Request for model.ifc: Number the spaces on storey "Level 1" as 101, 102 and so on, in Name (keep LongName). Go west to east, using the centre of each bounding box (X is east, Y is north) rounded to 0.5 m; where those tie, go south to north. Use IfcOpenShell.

First a look at what the model holds.

```python
import ifcopenshell
import ifcopenshell.util.element
import ifcopenshell.util.placement

model = ifcopenshell.open("model.ifc")
print(model.schema)
storey = next(s for s in model.by_type("IfcBuildingStorey") if s.Name == "Level 1")
spaces = [e for e in ifcopenshell.util.element.get_decomposition(storey) if e.is_a("IfcSpace")]
for e in sorted(spaces, key=lambda e: e.id()):
    origin = ifcopenshell.util.placement.get_local_placement(e.ObjectPlacement)[:3, 3]
    print(e.id(), e.Name, e.LongName, origin.round(2) + 0.0, sep=" | ")
```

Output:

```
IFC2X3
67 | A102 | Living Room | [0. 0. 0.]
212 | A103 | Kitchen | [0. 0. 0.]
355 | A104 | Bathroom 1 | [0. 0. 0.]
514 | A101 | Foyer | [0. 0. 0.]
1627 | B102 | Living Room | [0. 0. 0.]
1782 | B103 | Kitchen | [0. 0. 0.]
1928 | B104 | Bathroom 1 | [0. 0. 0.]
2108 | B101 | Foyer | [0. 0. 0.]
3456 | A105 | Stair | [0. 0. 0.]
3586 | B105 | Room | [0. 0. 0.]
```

```python
import ifcopenshell
import ifcopenshell.geom
import ifcopenshell.util.element
import ifcopenshell.util.shape

model = ifcopenshell.open("model.ifc")
settings = ifcopenshell.geom.settings()
settings.set("use-world-coords", True)


def centre(element):
    shape = ifcopenshell.geom.create_shape(settings, element)
    return ifcopenshell.util.shape.get_bbox_centroid(shape.geometry)


storey = next(s for s in model.by_type("IfcBuildingStorey") if s.Name == "Level 1")
spaces = [e for e in ifcopenshell.util.element.get_decomposition(storey) if e.is_a("IfcSpace")]

# Insertion points can sit at a corner or the storey origin, so sort by the geometry (in metres).
centres = {e: centre(e) for e in spaces}
spaces.sort(key=lambda e: (round(centres[e][0] / 0.5), centres[e][1]))

for i, e in enumerate(spaces, start=1):
    number = f"1{i:02d}"
    e.Name = number
    print(e.id(), number)

model.write("model_updated.ifc")
```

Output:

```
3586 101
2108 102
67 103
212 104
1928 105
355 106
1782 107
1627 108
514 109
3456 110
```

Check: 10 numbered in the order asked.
